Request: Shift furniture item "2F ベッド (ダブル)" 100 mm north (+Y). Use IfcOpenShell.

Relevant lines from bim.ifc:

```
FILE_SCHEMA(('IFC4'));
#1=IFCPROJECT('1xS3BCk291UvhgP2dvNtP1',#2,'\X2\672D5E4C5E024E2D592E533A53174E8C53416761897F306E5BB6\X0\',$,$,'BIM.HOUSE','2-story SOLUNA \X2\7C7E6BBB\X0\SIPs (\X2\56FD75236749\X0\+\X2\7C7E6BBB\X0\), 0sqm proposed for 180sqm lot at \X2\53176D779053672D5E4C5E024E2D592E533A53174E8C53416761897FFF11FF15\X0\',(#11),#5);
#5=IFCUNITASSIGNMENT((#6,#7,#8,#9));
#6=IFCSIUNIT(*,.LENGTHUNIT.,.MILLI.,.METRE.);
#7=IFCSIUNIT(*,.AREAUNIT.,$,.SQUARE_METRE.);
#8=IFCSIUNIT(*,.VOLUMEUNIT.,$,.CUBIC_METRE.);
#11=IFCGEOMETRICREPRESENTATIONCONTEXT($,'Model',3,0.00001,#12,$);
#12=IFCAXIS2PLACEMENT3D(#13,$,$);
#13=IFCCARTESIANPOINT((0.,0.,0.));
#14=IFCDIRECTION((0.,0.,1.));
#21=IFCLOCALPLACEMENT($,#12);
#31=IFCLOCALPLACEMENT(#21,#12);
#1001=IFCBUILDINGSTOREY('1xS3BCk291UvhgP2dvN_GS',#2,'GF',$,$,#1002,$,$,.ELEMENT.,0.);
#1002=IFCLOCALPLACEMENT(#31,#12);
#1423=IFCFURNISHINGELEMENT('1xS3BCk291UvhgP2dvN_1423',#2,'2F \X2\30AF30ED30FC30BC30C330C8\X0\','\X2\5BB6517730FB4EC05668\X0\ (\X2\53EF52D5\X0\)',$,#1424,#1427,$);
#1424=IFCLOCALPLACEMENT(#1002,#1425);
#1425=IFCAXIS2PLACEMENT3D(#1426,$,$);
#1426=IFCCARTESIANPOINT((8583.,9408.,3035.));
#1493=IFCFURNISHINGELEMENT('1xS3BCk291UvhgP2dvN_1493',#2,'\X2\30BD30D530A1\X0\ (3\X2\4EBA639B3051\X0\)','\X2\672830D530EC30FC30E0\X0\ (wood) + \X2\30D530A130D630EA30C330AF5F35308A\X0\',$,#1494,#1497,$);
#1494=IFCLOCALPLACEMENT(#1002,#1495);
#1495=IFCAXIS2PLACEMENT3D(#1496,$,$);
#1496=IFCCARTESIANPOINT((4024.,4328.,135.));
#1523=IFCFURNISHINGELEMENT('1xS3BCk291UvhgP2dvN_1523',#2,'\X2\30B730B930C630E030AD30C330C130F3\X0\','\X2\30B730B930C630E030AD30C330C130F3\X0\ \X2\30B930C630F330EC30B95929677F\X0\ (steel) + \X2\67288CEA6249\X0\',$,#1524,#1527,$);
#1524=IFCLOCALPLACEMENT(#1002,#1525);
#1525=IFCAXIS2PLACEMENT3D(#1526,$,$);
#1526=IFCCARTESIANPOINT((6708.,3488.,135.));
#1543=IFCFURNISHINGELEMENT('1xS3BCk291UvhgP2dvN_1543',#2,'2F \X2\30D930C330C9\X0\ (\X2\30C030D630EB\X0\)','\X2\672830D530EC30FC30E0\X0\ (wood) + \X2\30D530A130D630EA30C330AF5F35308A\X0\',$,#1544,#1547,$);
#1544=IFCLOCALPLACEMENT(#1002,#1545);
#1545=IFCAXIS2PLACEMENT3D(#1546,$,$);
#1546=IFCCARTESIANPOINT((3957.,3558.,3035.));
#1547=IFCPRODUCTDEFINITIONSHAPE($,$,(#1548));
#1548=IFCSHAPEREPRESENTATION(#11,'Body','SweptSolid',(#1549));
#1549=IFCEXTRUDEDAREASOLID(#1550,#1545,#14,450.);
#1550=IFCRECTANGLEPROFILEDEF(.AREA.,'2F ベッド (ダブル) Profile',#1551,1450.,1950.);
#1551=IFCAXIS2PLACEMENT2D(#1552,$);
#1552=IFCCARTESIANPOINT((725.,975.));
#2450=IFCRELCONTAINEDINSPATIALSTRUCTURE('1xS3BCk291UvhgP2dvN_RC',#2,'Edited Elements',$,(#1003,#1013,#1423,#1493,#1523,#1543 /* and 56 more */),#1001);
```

```python
import ifcopenshell
import ifcopenshell.api.geometry
import ifcopenshell.util.placement
import ifcopenshell.util.unit

model = ifcopenshell.open("bim.ifc")
unit_scale = ifcopenshell.util.unit.calculate_unit_scale(model)

item = model.by_id(1543)
matrix = ifcopenshell.util.placement.get_local_placement(item.ObjectPlacement)
matrix[1, 3] += 0.1 / unit_scale
ifcopenshell.api.geometry.edit_object_placement(model, product=item, matrix=matrix, is_si=False)

print(ifcopenshell.util.placement.get_local_placement(item.ObjectPlacement).round(3) + 0.0)

model.write("bim-out.ifc")
```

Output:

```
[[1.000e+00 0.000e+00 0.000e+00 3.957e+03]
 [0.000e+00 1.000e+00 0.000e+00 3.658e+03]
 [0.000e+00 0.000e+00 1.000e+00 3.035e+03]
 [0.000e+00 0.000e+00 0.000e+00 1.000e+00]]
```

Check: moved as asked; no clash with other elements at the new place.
